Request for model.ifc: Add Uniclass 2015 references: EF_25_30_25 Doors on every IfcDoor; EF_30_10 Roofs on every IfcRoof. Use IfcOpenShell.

First a look at what the model holds.

```python
import ifcopenshell

model = ifcopenshell.open("model.ifc")
print(model.schema)
print("classifications:", [c.Name for c in model.by_type("IfcClassification")])
for ifc_class in ("IfcDoor", "IfcRoof", "IfcStair", "IfcWall", "IfcWindow"):
    print(ifc_class, len(model.by_type(ifc_class)))
```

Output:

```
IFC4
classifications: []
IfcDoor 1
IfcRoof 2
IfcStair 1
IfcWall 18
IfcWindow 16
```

```python
import ifcopenshell
import ifcopenshell.api.classification

model = ifcopenshell.open("model.ifc")

system = ifcopenshell.api.classification.add_classification(model, classification="Uniclass 2015")

codes = {
    "IfcDoor": ("EF_25_30_25", "Doors"),
    "IfcRoof": ("EF_30_10", "Roofs"),
}
for ifc_class, (code, name) in codes.items():
    products = model.by_type(ifc_class)
    ifcopenshell.api.classification.add_reference(
        model, products=products, classification=system, identification=code, name=name
    )
    print(code, len(products))

model.write("model_updated.ifc")
```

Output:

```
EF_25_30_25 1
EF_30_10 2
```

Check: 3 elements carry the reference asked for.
